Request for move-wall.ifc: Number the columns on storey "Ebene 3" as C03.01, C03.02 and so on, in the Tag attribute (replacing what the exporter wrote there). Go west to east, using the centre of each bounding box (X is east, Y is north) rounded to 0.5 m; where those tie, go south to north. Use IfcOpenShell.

First a look at what the model holds.

```python
import ifcopenshell
import ifcopenshell.util.element
import ifcopenshell.util.placement

model = ifcopenshell.open("move-wall.ifc")
print(model.schema)
storey = next(s for s in model.by_type("IfcBuildingStorey") if s.Name == "Ebene 3")
columns = [e for e in ifcopenshell.util.element.get_decomposition(storey) if e.is_a("IfcColumn")]
for e in sorted(columns, key=lambda e: e.id()):
    origin = ifcopenshell.util.placement.get_local_placement(e.ObjectPlacement)[:3, 3]
    print(e.id(), e.Tag, e.Name, origin.round(2) + 0.0, sep=" | ")
```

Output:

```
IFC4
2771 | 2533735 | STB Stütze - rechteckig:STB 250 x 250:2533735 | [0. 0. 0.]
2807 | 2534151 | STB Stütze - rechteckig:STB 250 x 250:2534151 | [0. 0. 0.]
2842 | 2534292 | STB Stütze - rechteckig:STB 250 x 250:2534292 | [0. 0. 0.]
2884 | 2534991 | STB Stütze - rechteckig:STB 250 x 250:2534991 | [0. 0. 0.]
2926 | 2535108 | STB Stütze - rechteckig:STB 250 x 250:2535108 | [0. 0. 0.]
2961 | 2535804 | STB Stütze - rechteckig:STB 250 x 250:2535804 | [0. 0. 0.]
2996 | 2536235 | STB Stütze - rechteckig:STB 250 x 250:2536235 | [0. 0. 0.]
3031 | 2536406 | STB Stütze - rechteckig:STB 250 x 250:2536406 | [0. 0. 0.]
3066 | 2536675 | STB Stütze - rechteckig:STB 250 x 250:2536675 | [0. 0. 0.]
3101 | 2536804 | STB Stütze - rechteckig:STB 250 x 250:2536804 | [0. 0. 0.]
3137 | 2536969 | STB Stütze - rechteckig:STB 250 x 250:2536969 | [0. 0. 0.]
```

```python
import ifcopenshell
import ifcopenshell.geom
import ifcopenshell.util.element
import ifcopenshell.util.shape

model = ifcopenshell.open("move-wall.ifc")
settings = ifcopenshell.geom.settings()
settings.set("use-world-coords", True)


def centre(element):
    shape = ifcopenshell.geom.create_shape(settings, element)
    return ifcopenshell.util.shape.get_bbox_centroid(shape.geometry)


storey = next(s for s in model.by_type("IfcBuildingStorey") if s.Name == "Ebene 3")
columns = [e for e in ifcopenshell.util.element.get_decomposition(storey) if e.is_a("IfcColumn")]

# Insertion points can sit at a corner or the storey origin, so sort by the geometry (in metres).
centres = {e: centre(e) for e in columns}
columns.sort(key=lambda e: (round(centres[e][0] / 0.5), centres[e][1]))

for i, e in enumerate(columns, start=1):
    number = f"C03.{i:02d}"
    e.Tag = number
    print(e.id(), number)

model.write("move-wall_edited.ifc")
```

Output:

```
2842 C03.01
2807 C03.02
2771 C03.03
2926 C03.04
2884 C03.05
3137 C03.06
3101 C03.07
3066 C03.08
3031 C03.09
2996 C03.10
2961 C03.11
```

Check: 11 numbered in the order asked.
